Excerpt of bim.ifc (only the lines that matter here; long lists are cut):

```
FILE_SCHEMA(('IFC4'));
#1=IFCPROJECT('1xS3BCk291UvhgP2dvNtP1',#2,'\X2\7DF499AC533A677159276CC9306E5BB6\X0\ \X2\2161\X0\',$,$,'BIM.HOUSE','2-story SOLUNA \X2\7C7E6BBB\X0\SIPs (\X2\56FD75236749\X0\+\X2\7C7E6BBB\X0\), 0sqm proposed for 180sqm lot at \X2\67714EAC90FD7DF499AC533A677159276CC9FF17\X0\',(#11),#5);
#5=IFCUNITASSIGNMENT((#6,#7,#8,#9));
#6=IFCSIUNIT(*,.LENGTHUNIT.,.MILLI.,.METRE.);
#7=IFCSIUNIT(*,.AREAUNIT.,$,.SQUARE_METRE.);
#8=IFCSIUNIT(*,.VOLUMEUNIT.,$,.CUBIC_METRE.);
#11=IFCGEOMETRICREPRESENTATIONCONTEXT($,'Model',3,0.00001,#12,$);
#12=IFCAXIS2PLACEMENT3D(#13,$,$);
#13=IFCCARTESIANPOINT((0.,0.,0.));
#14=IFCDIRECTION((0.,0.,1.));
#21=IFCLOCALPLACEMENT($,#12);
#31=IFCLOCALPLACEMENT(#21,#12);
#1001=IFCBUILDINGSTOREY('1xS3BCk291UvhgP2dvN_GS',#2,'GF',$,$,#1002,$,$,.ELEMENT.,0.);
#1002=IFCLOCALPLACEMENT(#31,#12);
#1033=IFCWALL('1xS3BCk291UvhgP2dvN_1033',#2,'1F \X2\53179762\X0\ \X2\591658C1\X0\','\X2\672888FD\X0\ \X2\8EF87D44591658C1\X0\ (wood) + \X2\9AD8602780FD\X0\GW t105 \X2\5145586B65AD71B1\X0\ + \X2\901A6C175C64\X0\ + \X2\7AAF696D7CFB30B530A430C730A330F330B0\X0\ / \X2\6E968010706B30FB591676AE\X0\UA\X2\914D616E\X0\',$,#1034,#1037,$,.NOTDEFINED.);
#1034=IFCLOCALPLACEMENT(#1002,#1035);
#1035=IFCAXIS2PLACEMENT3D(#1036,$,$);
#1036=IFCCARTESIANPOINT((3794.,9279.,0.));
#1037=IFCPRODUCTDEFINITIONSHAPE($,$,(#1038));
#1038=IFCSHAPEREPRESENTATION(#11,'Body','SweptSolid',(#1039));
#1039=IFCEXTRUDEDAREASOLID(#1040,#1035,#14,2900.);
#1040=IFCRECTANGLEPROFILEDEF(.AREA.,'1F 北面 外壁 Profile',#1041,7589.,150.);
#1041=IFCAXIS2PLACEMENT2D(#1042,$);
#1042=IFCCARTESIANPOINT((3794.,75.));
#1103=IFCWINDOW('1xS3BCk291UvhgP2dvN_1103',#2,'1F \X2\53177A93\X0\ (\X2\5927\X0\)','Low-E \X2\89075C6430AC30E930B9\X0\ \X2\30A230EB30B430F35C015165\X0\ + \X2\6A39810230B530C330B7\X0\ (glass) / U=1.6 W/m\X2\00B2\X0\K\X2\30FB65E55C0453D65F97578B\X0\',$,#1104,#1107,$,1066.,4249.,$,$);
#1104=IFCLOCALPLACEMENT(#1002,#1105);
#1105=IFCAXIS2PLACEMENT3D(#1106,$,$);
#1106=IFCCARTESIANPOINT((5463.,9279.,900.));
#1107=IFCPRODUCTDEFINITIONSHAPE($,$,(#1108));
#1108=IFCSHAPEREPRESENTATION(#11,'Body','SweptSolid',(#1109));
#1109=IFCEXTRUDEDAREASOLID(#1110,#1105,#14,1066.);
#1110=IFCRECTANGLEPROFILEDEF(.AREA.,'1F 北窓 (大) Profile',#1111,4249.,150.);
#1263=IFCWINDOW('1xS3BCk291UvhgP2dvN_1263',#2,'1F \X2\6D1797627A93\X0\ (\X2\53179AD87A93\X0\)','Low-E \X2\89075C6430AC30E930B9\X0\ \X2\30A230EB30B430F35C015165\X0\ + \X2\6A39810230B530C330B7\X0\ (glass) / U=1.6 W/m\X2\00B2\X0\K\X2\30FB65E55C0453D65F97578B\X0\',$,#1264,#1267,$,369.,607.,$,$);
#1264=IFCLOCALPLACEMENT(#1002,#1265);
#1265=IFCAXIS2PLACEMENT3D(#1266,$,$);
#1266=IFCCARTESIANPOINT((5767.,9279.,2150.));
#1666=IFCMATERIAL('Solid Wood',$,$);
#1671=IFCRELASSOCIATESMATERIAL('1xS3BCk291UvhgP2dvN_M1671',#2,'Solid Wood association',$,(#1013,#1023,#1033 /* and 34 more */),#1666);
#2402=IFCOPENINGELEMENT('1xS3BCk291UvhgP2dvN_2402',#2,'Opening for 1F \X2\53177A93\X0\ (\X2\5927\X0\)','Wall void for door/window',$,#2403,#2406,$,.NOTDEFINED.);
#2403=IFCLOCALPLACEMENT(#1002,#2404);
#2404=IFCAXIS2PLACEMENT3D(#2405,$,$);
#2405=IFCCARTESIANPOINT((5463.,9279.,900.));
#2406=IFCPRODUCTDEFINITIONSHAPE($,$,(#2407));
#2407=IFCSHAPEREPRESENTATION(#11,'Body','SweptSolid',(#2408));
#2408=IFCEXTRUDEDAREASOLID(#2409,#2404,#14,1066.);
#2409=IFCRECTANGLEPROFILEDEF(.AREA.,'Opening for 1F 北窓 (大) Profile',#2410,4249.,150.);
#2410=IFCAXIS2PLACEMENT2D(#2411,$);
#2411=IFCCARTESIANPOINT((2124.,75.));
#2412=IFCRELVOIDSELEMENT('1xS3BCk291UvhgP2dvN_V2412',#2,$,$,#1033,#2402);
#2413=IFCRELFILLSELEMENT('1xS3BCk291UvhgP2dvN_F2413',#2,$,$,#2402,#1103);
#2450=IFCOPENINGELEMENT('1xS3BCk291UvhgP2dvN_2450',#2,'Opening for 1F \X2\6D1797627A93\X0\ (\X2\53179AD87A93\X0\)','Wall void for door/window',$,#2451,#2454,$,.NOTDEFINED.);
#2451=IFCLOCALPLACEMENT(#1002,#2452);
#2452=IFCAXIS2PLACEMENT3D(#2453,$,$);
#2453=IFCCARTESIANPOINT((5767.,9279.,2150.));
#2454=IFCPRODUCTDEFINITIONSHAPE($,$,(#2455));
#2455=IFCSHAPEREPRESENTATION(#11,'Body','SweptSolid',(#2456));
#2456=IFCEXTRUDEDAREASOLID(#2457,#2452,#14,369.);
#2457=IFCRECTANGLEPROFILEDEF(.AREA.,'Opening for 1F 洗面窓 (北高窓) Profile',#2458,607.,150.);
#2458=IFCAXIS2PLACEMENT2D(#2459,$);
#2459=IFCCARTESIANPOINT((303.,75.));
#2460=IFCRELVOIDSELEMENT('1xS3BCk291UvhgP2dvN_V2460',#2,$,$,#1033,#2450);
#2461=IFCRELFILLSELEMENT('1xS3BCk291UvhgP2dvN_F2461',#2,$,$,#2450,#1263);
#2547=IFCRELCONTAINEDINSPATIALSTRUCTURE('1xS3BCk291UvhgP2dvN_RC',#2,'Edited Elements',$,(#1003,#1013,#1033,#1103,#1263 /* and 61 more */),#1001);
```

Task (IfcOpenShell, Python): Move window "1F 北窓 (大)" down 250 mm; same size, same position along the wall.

```python
import numpy as np
import ifcopenshell
import ifcopenshell.api.geometry
import ifcopenshell.util.placement
import ifcopenshell.util.unit

model = ifcopenshell.open("bim.ifc")
unit_scale = ifcopenshell.util.unit.calculate_unit_scale(model)

window = model.by_guid("1xS3BCk291UvhgP2dvN_1103")
opening = window.FillsVoids[0].RelatingOpeningElement
dz = -0.25 / unit_scale

shift = np.array([0.0, 0.0, dz])
# The window is not placed relative to its opening, so move both.
for product in (opening, window):
    matrix = ifcopenshell.util.placement.get_local_placement(product.ObjectPlacement)
    matrix[:3, 3] += shift
    ifcopenshell.api.geometry.edit_object_placement(model, product=product, matrix=matrix, is_si=False)

print(f"moved by {dz * unit_scale:+.3f} m")

model.write("bim_rev.ifc")
```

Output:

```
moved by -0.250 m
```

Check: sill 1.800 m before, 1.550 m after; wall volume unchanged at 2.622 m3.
